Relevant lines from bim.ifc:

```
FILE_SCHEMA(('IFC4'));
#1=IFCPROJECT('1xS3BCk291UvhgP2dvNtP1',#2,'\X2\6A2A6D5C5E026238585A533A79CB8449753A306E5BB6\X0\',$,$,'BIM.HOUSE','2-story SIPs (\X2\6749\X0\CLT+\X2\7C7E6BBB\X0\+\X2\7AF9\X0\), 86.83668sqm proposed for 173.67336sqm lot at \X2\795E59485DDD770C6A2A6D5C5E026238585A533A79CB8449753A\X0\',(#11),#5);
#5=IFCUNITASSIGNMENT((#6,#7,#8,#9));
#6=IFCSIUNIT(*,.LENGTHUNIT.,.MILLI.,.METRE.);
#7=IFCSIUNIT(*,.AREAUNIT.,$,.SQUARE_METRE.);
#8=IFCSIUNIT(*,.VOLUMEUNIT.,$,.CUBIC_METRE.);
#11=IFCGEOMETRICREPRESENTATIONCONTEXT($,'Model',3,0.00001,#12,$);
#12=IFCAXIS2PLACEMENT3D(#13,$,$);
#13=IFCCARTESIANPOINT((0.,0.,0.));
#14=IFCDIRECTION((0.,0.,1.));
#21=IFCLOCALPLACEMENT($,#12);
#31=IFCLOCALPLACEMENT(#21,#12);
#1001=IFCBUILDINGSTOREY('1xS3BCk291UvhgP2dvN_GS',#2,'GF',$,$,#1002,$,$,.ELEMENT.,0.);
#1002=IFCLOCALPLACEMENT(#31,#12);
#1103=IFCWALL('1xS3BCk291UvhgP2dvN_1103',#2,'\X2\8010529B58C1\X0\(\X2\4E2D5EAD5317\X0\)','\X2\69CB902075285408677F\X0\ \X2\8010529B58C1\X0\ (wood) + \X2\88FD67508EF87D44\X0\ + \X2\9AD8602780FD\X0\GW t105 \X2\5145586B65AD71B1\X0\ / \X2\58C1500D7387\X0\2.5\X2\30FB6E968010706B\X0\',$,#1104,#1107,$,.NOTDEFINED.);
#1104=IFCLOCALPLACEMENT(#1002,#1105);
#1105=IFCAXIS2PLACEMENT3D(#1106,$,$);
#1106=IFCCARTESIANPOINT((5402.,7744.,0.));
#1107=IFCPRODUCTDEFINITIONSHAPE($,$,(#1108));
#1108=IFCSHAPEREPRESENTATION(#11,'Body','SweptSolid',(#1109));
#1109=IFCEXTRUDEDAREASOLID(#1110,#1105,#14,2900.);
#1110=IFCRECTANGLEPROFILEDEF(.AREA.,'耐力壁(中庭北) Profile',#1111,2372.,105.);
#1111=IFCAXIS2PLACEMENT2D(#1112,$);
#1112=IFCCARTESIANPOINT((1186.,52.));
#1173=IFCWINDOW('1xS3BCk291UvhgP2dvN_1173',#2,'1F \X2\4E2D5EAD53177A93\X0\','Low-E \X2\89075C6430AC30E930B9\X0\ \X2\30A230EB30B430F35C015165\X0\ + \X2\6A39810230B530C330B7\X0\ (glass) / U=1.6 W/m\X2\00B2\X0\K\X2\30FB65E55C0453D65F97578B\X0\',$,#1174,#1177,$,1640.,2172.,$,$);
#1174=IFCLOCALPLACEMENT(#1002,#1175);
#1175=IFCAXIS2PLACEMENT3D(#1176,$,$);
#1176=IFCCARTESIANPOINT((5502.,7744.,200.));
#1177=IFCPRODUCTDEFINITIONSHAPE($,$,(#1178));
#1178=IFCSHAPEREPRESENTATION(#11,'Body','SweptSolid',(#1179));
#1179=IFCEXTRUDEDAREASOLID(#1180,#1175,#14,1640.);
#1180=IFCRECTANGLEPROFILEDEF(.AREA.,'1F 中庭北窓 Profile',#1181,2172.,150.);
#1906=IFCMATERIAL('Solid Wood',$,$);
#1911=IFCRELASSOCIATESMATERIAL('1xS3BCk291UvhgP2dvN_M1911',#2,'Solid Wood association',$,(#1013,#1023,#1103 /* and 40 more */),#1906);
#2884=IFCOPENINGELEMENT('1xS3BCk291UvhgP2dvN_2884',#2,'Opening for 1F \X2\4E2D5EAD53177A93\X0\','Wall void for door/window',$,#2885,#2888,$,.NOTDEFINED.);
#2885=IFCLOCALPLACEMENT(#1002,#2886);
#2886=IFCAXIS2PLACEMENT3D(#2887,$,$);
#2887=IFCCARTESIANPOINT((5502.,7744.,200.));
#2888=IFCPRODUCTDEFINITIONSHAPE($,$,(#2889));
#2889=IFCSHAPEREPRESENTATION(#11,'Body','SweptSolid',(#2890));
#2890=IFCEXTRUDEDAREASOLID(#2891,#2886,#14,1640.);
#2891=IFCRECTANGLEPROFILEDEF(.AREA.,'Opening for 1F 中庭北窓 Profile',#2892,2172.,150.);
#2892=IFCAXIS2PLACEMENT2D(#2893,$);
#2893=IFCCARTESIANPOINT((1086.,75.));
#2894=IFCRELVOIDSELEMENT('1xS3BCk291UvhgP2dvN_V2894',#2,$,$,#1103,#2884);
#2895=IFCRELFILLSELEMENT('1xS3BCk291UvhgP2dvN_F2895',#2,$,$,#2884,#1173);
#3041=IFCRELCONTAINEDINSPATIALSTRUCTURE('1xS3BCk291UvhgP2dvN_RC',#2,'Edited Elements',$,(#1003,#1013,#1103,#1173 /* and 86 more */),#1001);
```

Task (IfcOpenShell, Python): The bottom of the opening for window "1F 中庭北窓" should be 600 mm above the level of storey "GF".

```python
import numpy as np
import ifcopenshell
import ifcopenshell.api.geometry
import ifcopenshell.geom
import ifcopenshell.util.element
import ifcopenshell.util.placement
import ifcopenshell.util.shape
import ifcopenshell.util.unit

model = ifcopenshell.open("bim.ifc")
unit_scale = ifcopenshell.util.unit.calculate_unit_scale(model)

window = model.by_guid("1xS3BCk291UvhgP2dvN_1173")
opening = window.FillsVoids[0].RelatingOpeningElement
storey = ifcopenshell.util.element.get_container(window, ifc_class="IfcBuildingStorey")
level = ifcopenshell.util.placement.get_local_placement(storey.ObjectPlacement)[2, 3]

# The opening's origin need not be at the sill, so measure its lowest point.
shape = ifcopenshell.geom.create_shape(ifcopenshell.geom.settings(), opening)
bottom = ifcopenshell.util.shape.get_shape_bottom_elevation(shape, shape.geometry) / unit_scale
dz = level + 600.0 - bottom

shift = np.array([0.0, 0.0, dz])
# The window is not placed relative to its opening, so move both.
for product in (opening, window):
    matrix = ifcopenshell.util.placement.get_local_placement(product.ObjectPlacement)
    matrix[:3, 3] += shift
    ifcopenshell.api.geometry.edit_object_placement(model, product=product, matrix=matrix, is_si=False)

print(f"moved by {dz * unit_scale:+.3f} m")

model.write("bim_edited.ifc")
```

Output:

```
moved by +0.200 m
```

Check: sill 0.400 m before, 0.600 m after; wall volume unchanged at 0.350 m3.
